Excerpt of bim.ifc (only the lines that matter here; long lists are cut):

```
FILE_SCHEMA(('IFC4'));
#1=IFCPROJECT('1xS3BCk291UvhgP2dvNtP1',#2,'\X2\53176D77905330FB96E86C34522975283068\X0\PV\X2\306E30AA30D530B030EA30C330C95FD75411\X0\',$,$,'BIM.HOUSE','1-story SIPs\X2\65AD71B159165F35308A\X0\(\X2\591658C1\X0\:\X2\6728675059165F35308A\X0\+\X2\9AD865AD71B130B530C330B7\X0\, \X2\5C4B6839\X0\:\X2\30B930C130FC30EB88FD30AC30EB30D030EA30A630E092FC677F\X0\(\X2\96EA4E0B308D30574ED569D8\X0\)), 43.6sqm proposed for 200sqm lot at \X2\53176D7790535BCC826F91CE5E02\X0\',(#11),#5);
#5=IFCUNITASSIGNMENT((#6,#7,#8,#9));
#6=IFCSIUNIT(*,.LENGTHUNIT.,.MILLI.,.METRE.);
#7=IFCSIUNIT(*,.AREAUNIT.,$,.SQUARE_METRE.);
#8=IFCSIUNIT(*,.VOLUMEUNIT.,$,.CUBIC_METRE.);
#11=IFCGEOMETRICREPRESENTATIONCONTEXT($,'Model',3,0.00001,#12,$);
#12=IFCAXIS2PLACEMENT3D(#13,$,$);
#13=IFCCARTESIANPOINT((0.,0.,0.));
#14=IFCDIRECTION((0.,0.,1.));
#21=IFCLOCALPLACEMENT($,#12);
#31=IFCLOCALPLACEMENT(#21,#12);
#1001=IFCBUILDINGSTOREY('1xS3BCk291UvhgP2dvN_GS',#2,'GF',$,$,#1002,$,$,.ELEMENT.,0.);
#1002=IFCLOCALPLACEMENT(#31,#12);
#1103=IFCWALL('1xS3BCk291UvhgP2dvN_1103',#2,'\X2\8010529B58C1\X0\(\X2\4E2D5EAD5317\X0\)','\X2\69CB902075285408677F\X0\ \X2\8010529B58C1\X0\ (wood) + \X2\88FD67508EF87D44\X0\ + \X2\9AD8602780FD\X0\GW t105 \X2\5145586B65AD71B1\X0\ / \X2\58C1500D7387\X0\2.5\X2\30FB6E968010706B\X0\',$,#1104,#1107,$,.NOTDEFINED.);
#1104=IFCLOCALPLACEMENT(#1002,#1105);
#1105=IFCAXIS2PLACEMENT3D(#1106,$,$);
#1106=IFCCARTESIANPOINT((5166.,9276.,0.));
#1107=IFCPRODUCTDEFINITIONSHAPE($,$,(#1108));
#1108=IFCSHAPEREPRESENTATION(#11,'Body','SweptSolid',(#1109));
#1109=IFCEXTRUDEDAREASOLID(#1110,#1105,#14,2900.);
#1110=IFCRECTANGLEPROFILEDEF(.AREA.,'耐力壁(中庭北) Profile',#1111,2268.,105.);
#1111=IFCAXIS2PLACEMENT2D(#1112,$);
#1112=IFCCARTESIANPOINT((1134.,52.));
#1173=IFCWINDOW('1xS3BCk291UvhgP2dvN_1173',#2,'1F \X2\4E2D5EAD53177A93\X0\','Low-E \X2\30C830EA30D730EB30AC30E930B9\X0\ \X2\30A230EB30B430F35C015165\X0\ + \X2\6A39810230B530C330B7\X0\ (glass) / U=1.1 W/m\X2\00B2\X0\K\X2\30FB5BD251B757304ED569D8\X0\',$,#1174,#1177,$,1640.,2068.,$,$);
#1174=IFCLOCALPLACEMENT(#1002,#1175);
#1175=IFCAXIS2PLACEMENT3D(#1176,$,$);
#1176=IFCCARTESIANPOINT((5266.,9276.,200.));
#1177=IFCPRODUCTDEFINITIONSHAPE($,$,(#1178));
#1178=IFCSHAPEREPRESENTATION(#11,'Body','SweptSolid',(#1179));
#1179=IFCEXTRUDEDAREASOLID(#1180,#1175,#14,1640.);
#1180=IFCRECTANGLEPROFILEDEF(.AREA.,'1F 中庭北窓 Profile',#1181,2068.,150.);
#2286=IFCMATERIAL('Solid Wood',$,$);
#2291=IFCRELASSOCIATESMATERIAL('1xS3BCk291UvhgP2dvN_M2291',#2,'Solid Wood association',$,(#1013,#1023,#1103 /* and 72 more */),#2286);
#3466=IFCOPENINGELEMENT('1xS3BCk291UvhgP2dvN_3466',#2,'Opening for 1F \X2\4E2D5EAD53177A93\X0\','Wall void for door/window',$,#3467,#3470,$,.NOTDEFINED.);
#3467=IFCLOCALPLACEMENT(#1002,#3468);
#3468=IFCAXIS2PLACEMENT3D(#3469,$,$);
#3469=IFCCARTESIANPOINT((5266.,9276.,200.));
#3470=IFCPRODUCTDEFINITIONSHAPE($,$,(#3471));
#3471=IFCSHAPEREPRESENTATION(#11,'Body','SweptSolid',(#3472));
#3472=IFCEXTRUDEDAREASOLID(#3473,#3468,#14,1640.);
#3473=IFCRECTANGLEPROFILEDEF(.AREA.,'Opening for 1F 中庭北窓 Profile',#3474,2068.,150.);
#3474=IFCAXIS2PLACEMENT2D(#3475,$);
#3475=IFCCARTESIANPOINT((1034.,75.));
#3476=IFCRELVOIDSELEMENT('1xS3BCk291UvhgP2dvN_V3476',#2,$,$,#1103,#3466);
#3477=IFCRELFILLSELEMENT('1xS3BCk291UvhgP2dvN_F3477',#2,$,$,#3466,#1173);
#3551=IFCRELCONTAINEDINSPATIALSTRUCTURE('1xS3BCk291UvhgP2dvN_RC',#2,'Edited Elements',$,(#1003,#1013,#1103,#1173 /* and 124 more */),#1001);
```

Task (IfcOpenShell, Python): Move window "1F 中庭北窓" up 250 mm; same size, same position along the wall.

```python
import numpy as np
import ifcopenshell
import ifcopenshell.api.geometry
import ifcopenshell.util.placement
import ifcopenshell.util.unit

model = ifcopenshell.open("bim.ifc")
unit_scale = ifcopenshell.util.unit.calculate_unit_scale(model)

window = model.by_id(1173)
opening = window.FillsVoids[0].RelatingOpeningElement
dz = 250.0

shift = np.array([0.0, 0.0, dz])
# The window is not placed relative to its opening, so move both.
for product in (opening, window):
    matrix = ifcopenshell.util.placement.get_local_placement(product.ObjectPlacement)
    matrix[:3, 3] += shift
    ifcopenshell.api.geometry.edit_object_placement(model, product=product, matrix=matrix, is_si=False)

print(f"moved by {dz * unit_scale:+.3f} m")

model.write("bim_rev.ifc")
```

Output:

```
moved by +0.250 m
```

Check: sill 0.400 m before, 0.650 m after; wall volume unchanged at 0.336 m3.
